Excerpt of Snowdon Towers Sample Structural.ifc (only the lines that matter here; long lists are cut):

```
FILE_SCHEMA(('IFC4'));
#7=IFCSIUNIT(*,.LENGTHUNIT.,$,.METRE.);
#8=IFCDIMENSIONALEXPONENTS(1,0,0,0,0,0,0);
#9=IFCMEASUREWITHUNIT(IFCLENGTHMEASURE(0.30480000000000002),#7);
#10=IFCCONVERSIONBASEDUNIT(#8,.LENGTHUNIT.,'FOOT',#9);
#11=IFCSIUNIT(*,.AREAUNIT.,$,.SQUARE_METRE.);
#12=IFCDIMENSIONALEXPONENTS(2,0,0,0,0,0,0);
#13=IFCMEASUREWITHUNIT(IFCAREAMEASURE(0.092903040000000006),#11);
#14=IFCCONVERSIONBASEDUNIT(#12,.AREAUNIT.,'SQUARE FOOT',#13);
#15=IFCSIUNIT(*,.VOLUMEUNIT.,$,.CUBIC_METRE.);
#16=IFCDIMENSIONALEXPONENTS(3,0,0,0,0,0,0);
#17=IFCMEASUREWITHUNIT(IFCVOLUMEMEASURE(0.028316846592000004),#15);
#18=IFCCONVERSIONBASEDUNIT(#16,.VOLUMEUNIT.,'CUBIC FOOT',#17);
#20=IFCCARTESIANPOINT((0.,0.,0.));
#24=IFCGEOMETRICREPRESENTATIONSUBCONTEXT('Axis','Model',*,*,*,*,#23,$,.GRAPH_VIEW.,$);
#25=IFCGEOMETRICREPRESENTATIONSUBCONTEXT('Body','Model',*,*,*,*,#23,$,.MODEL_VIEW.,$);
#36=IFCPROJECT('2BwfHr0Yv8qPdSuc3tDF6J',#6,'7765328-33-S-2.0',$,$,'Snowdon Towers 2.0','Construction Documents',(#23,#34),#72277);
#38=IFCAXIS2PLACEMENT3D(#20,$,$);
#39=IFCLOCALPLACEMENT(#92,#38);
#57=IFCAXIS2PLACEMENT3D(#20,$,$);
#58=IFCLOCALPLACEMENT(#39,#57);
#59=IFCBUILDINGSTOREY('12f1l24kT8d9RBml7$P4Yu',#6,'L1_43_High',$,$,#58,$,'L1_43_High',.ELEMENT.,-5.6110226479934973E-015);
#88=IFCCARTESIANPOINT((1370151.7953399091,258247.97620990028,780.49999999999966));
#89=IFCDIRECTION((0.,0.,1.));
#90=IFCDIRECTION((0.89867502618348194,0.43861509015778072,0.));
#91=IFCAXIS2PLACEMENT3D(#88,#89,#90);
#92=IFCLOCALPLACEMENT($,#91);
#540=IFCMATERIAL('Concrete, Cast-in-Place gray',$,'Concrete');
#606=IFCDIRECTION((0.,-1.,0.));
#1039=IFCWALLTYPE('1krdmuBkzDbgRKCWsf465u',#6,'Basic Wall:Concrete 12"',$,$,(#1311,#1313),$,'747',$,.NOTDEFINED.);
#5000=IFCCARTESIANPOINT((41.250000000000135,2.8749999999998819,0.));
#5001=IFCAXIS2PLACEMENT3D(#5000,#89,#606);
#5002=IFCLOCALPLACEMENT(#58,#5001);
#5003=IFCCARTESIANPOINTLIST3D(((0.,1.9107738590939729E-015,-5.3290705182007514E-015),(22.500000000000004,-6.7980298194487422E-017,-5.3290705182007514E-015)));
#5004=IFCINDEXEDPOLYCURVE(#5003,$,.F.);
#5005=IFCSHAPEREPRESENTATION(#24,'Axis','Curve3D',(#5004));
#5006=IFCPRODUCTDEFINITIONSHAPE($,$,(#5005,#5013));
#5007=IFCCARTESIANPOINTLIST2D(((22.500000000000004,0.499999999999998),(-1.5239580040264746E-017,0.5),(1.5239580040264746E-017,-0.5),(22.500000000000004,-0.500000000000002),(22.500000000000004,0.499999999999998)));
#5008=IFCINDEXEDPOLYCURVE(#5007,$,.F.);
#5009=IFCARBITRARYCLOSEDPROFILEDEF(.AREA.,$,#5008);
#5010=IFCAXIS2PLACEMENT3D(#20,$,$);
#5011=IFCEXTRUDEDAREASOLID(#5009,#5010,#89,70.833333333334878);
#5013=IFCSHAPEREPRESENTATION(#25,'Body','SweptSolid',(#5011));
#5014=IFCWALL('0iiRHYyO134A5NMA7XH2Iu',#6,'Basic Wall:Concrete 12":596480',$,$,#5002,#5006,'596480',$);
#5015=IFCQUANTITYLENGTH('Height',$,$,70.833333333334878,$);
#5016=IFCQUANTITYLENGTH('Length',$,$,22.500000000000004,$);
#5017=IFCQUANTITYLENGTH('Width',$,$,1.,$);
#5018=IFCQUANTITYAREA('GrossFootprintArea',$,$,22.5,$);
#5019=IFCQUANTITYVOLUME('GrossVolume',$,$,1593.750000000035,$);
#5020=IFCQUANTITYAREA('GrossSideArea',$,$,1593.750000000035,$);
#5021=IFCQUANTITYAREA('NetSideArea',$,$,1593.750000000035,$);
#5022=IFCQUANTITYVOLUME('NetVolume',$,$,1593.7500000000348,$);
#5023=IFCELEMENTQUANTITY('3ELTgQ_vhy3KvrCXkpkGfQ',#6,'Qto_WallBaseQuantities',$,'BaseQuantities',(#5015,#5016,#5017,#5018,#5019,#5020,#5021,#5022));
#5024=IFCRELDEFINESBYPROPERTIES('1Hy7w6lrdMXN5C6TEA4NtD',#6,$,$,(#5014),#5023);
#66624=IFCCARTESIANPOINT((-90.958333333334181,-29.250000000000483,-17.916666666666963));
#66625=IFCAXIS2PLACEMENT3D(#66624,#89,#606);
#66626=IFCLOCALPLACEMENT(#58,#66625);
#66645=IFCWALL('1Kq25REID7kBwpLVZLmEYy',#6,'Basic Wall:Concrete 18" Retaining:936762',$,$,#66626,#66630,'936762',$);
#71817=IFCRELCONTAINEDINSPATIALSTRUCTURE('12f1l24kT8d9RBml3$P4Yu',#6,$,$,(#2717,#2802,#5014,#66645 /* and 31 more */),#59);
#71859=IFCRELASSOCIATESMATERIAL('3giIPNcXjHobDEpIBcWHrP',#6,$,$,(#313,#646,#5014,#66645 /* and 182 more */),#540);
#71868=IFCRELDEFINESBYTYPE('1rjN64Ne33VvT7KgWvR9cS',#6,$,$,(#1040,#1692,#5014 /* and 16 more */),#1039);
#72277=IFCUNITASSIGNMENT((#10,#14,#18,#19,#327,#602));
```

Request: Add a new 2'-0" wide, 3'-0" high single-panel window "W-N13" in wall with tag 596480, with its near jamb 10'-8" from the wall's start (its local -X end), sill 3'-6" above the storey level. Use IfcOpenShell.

```python
import numpy as np
import ifcopenshell
import ifcopenshell.api.feature
import ifcopenshell.api.geometry
import ifcopenshell.api.pset
import ifcopenshell.api.root
import ifcopenshell.api.spatial
import ifcopenshell.geom
import ifcopenshell.util.element
import ifcopenshell.util.placement
import ifcopenshell.util.representation
import ifcopenshell.util.shape
import ifcopenshell.util.unit

model = ifcopenshell.open("Snowdon Towers Sample Structural.ifc")
unit_scale = ifcopenshell.util.unit.calculate_unit_scale(model)
area_scale = ifcopenshell.util.unit.calculate_unit_scale(model, "AREAUNIT")
volume_scale = ifcopenshell.util.unit.calculate_unit_scale(model, "VOLUMEUNIT")
settings = ifcopenshell.geom.settings()


def volume(element):
    """Net volume in cubic metres, openings subtracted."""
    shape = ifcopenshell.geom.create_shape(settings, element)
    return ifcopenshell.util.shape.get_volume(shape.geometry)


wall = model.by_guid("0iiRHYyO134A5NMA7XH2Iu")
storey = ifcopenshell.util.element.get_container(wall, ifc_class="IfcBuildingStorey")
context = ifcopenshell.util.representation.get_context(model, "Model", "Body", "MODEL_VIEW")
before = volume(wall)

width, height, from_end, sill = 0.6096, 0.9144, 3.2512, 1.0668  # metres

# The wall runs along its own X axis, and the end named is its -X end.
wall_shape = ifcopenshell.geom.create_shape(settings, wall)
x, y, z = ifcopenshell.util.shape.get_vertices(wall_shape.geometry).T
start = x.min() + from_end
face, thickness = float(y.min()), float(y.max() - y.min())
wall_matrix = ifcopenshell.util.placement.get_local_placement(wall.ObjectPlacement)
level = ifcopenshell.util.placement.get_local_placement(storey.ObjectPlacement)[2, 3]


def in_wall(x, y):
    """Placement at x, y metres in the wall's axes, at sill height."""
    matrix = wall_matrix.copy()
    matrix[:, 3] = wall_matrix @ np.array([x / unit_scale, y / unit_scale, 0.0, 1.0])
    matrix[2, 3] = level + sill / unit_scale
    return matrix


# Opening: a box that overshoots both wall faces by 50 mm.
opening = ifcopenshell.api.root.create_entity(model, ifc_class="IfcOpeningElement", predefined_type="OPENING")
box = ifcopenshell.api.geometry.add_wall_representation(
    model, context=context, length=width, height=height, thickness=thickness + 0.1
)
ifcopenshell.api.geometry.assign_representation(model, product=opening, representation=box)
ifcopenshell.api.geometry.edit_object_placement(model, product=opening, matrix=in_wall(start, face - 0.05), is_si=False)
ifcopenshell.api.feature.add_feature(model, feature=opening, element=wall)

window = ifcopenshell.api.root.create_entity(model, ifc_class="IfcWindow", name="W-N13", predefined_type="WINDOW")
window.OverallWidth, window.OverallHeight = width / unit_scale, height / unit_scale
window.PartitioningType = "SINGLE_PANEL"
body = ifcopenshell.api.geometry.add_window_representation(
    model,
    context=context,
    overall_width=window.OverallWidth,
    overall_height=window.OverallHeight,
    partition_type="SINGLE_PANEL",
)
ifcopenshell.api.geometry.assign_representation(model, product=window, representation=body)
ifcopenshell.api.spatial.assign_container(model, products=[window], relating_structure=storey)
ifcopenshell.api.feature.add_filling(model, opening=opening, element=window)

# Centre the window in the wall's thickness.
ifcopenshell.api.geometry.edit_object_placement(model, product=window, matrix=in_wall(start, face), is_si=False)
window_shape = ifcopenshell.geom.create_shape(settings, window)
depth = ifcopenshell.util.shape.get_vertices(window_shape.geometry)[:, 1]
offset = face + thickness / 2 - (depth.min() + depth.max()) / 2
ifcopenshell.api.geometry.edit_object_placement(model, product=window, matrix=in_wall(start, offset), is_si=False)

after = volume(wall)

# Update the wall's stored quantities.
qto = model.by_id(ifcopenshell.util.element.get_pset(wall, "Qto_WallBaseQuantities", should_inherit=False)["id"])
ifcopenshell.api.pset.edit_qto(model, qto=qto, properties={
    "NetSideArea": after / thickness / area_scale,
    "NetVolume": after / volume_scale,
})

print(f"wall volume {before:.3f} -> {after:.3f} m3")

model.write("Snowdon Towers Sample Structural_updated.ifc")
```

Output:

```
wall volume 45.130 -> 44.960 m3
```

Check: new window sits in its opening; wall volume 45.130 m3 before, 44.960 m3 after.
